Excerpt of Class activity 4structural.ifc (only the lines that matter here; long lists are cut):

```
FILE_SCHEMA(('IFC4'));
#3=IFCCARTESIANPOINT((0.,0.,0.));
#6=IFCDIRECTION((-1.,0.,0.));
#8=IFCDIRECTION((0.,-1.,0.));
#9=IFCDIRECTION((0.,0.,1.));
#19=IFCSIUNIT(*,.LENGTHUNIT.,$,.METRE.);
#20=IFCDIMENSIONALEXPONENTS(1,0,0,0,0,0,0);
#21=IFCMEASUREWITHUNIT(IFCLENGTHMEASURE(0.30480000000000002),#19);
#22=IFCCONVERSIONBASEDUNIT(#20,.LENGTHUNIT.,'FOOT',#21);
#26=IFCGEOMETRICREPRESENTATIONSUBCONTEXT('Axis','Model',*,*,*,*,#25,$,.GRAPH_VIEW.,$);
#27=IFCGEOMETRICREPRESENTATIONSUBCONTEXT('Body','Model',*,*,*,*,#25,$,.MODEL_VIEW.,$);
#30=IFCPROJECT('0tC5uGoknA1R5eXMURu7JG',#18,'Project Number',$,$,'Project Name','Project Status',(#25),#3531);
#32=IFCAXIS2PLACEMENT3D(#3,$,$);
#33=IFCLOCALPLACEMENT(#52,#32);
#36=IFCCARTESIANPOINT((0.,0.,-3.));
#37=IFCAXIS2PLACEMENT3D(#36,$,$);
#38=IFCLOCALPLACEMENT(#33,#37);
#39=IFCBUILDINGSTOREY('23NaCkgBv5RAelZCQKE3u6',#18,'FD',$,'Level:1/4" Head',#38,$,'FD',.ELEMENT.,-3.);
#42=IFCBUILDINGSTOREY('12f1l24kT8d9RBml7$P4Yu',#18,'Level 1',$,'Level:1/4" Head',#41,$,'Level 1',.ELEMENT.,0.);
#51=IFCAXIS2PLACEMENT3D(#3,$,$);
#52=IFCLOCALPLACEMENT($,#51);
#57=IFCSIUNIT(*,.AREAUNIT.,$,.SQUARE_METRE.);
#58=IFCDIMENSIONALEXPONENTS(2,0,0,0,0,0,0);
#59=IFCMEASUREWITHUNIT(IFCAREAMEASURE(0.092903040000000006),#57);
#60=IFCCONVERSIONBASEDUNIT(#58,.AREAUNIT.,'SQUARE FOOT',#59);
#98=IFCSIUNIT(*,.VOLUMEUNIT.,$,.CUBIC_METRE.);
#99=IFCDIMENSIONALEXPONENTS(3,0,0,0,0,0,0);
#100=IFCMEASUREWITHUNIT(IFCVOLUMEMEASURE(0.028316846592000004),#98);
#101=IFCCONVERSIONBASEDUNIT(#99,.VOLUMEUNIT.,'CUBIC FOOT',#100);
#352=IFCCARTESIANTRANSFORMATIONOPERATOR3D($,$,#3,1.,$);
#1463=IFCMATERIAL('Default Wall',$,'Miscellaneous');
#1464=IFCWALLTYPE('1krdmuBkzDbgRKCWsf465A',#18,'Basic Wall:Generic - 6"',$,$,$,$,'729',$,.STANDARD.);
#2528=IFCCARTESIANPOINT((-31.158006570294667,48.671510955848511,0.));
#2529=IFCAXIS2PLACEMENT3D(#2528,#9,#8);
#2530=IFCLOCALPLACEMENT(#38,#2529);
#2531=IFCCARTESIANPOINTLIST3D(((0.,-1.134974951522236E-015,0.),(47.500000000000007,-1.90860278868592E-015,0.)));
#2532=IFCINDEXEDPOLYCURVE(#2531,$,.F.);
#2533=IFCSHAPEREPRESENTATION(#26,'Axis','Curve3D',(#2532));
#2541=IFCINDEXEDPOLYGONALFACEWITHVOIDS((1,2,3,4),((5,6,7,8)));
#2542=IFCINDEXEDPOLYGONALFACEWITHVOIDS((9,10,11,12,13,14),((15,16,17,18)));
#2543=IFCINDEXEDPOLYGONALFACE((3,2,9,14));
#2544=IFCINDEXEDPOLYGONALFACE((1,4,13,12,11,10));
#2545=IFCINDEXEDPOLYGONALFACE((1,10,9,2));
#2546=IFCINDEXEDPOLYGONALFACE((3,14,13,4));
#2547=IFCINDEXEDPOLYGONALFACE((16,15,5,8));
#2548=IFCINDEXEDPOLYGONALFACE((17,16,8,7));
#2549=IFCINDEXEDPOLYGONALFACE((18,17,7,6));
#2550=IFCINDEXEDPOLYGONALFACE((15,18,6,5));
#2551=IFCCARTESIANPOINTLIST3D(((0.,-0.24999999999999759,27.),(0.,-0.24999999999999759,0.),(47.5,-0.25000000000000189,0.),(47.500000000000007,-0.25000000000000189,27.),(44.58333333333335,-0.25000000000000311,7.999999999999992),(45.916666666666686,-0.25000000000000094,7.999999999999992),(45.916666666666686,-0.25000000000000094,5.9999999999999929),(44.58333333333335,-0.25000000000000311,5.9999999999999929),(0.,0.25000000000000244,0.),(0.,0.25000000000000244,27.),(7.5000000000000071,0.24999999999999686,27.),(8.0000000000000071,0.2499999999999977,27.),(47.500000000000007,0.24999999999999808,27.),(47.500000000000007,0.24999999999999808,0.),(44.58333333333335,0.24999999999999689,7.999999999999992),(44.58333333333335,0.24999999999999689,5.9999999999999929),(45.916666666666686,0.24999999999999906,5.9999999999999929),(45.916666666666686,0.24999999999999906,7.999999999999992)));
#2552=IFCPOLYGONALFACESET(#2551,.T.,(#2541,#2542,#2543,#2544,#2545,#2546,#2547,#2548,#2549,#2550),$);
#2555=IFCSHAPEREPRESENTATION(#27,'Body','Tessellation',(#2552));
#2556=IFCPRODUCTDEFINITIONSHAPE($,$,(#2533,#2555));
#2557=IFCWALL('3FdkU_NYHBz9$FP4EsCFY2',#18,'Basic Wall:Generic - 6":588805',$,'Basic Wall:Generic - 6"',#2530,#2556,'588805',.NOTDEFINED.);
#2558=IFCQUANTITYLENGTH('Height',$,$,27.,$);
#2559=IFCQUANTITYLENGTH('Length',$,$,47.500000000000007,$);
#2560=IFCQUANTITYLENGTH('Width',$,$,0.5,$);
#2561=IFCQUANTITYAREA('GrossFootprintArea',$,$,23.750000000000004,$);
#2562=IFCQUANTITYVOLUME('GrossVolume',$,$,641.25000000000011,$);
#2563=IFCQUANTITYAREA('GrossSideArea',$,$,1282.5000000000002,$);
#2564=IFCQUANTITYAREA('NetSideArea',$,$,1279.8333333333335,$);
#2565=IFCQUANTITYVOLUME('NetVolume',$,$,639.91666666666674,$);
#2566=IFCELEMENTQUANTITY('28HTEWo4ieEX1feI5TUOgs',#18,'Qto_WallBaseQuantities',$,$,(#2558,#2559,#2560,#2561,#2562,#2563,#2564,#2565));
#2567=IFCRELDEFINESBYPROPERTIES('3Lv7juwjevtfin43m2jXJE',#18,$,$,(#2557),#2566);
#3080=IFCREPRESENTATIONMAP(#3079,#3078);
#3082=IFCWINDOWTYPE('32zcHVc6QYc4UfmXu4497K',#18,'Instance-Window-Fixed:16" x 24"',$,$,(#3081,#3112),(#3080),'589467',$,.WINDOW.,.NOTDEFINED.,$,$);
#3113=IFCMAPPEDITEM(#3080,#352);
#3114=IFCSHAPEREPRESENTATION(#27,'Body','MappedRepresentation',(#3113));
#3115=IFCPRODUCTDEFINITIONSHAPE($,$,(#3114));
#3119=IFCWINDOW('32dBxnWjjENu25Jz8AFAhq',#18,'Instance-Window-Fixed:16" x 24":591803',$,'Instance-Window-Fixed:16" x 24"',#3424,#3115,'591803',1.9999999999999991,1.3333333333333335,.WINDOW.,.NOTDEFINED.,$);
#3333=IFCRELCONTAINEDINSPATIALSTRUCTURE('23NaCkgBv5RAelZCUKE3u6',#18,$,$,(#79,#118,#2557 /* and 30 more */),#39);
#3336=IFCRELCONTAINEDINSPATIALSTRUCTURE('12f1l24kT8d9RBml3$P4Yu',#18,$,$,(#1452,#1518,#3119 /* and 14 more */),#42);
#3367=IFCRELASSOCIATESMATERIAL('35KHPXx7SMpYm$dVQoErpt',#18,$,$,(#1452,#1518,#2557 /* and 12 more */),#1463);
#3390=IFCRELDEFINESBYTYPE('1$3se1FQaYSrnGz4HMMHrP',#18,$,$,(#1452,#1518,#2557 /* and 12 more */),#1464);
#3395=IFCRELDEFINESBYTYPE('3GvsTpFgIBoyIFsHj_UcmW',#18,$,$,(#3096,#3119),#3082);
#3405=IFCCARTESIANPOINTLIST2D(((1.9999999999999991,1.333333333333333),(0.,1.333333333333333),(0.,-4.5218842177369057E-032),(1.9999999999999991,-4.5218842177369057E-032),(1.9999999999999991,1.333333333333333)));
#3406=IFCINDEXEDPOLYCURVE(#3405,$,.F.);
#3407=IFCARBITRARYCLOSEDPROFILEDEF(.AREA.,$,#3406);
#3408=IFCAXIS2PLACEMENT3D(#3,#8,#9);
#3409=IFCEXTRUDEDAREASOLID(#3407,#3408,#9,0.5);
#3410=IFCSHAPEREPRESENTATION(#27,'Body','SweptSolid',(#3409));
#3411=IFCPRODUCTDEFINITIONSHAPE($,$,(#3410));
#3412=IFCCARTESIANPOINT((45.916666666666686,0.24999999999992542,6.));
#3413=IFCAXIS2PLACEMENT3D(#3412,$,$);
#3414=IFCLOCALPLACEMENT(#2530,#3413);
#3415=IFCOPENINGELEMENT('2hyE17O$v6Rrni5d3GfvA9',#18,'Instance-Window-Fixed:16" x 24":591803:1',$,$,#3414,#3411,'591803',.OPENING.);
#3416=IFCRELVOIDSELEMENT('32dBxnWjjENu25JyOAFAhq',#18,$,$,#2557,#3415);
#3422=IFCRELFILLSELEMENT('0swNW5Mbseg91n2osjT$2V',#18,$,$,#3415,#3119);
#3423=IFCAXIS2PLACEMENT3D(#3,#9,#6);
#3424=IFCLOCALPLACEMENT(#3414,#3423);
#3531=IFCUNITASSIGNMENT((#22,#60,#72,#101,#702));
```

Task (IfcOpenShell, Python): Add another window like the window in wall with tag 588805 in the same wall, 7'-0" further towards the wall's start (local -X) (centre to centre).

```python
import ifcopenshell
import ifcopenshell.api.feature
import ifcopenshell.api.geometry
import ifcopenshell.api.pset
import ifcopenshell.api.root
import ifcopenshell.geom
import ifcopenshell.util.element
import ifcopenshell.util.placement
import ifcopenshell.util.shape
import ifcopenshell.util.unit

model = ifcopenshell.open("Class activity 4structural.ifc")
unit_scale = ifcopenshell.util.unit.calculate_unit_scale(model)
area_scale = ifcopenshell.util.unit.calculate_unit_scale(model, "AREAUNIT")
volume_scale = ifcopenshell.util.unit.calculate_unit_scale(model, "VOLUMEUNIT")
settings = ifcopenshell.geom.settings()


def volume(element):
    """Net volume in cubic metres, openings subtracted."""
    shape = ifcopenshell.geom.create_shape(settings, element)
    return ifcopenshell.util.shape.get_volume(shape.geometry)


def reuse_history(source, copy):
    """copy_class also copies each property set's owner history, people and application; keep the originals."""
    for rel in copy.IsDefinedBy:
        if rel.is_a("IfcRelDefinesByProperties") and (history := rel.RelatingPropertyDefinition.OwnerHistory):
            rel.RelatingPropertyDefinition.OwnerHistory = source.OwnerHistory
            ifcopenshell.util.element.remove_deep2(model, history)


window = model.by_guid("32dBxnWjjENu25Jz8AFAhq")
opening = window.FillsVoids[0].RelatingOpeningElement
wall = opening.VoidsElements[0].RelatingBuildingElement
before = volume(wall)
shift = ifcopenshell.util.placement.get_local_placement(wall.ObjectPlacement)[:3, 0] * -84 * 0.0254 / unit_scale

# copy_class copies the void relationship, type, container and properties, but no geometry.
new_opening = ifcopenshell.api.root.copy_class(model, product=opening)
new_opening.Representation = ifcopenshell.util.element.copy_deep(
    model, opening.Representation, exclude=["IfcGeometricRepresentationContext", "IfcRepresentationMap"]
)
new_opening.Name = 'Instance-Window-Fixed:16" x 24"'
new_opening.Tag = None
reuse_history(opening, new_opening)
new_window = ifcopenshell.api.root.copy_class(model, product=window)
new_window.Representation = ifcopenshell.util.element.copy_deep(
    model, window.Representation, exclude=["IfcGeometricRepresentationContext", "IfcRepresentationMap"]
)
new_window.Name = 'Instance-Window-Fixed:16" x 24"'
new_window.Tag = None
reuse_history(window, new_window)
ifcopenshell.api.feature.add_filling(model, opening=new_opening, element=new_window)

for old, new in ((opening, new_opening), (window, new_window)):
    matrix = ifcopenshell.util.placement.get_local_placement(old.ObjectPlacement)
    matrix[:3, 3] += shift
    ifcopenshell.api.geometry.edit_object_placement(model, product=new, matrix=matrix, is_si=False)

after = volume(wall)
thickness = 0.1524  # wall thickness in metres

# Update the wall's stored quantities.
qto = model.by_id(ifcopenshell.util.element.get_pset(wall, "Qto_WallBaseQuantities", should_inherit=False)["id"])
ifcopenshell.api.pset.edit_qto(model, qto=qto, properties={
    "NetSideArea": after / thickness / area_scale,
    "NetVolume": after / volume_scale,
})

print(f"wall volume {before:.3f} -> {after:.3f} m3")

model.write("Class activity 4structural_rev.ifc")
```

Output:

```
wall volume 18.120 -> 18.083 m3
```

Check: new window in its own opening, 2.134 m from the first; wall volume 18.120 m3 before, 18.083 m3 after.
